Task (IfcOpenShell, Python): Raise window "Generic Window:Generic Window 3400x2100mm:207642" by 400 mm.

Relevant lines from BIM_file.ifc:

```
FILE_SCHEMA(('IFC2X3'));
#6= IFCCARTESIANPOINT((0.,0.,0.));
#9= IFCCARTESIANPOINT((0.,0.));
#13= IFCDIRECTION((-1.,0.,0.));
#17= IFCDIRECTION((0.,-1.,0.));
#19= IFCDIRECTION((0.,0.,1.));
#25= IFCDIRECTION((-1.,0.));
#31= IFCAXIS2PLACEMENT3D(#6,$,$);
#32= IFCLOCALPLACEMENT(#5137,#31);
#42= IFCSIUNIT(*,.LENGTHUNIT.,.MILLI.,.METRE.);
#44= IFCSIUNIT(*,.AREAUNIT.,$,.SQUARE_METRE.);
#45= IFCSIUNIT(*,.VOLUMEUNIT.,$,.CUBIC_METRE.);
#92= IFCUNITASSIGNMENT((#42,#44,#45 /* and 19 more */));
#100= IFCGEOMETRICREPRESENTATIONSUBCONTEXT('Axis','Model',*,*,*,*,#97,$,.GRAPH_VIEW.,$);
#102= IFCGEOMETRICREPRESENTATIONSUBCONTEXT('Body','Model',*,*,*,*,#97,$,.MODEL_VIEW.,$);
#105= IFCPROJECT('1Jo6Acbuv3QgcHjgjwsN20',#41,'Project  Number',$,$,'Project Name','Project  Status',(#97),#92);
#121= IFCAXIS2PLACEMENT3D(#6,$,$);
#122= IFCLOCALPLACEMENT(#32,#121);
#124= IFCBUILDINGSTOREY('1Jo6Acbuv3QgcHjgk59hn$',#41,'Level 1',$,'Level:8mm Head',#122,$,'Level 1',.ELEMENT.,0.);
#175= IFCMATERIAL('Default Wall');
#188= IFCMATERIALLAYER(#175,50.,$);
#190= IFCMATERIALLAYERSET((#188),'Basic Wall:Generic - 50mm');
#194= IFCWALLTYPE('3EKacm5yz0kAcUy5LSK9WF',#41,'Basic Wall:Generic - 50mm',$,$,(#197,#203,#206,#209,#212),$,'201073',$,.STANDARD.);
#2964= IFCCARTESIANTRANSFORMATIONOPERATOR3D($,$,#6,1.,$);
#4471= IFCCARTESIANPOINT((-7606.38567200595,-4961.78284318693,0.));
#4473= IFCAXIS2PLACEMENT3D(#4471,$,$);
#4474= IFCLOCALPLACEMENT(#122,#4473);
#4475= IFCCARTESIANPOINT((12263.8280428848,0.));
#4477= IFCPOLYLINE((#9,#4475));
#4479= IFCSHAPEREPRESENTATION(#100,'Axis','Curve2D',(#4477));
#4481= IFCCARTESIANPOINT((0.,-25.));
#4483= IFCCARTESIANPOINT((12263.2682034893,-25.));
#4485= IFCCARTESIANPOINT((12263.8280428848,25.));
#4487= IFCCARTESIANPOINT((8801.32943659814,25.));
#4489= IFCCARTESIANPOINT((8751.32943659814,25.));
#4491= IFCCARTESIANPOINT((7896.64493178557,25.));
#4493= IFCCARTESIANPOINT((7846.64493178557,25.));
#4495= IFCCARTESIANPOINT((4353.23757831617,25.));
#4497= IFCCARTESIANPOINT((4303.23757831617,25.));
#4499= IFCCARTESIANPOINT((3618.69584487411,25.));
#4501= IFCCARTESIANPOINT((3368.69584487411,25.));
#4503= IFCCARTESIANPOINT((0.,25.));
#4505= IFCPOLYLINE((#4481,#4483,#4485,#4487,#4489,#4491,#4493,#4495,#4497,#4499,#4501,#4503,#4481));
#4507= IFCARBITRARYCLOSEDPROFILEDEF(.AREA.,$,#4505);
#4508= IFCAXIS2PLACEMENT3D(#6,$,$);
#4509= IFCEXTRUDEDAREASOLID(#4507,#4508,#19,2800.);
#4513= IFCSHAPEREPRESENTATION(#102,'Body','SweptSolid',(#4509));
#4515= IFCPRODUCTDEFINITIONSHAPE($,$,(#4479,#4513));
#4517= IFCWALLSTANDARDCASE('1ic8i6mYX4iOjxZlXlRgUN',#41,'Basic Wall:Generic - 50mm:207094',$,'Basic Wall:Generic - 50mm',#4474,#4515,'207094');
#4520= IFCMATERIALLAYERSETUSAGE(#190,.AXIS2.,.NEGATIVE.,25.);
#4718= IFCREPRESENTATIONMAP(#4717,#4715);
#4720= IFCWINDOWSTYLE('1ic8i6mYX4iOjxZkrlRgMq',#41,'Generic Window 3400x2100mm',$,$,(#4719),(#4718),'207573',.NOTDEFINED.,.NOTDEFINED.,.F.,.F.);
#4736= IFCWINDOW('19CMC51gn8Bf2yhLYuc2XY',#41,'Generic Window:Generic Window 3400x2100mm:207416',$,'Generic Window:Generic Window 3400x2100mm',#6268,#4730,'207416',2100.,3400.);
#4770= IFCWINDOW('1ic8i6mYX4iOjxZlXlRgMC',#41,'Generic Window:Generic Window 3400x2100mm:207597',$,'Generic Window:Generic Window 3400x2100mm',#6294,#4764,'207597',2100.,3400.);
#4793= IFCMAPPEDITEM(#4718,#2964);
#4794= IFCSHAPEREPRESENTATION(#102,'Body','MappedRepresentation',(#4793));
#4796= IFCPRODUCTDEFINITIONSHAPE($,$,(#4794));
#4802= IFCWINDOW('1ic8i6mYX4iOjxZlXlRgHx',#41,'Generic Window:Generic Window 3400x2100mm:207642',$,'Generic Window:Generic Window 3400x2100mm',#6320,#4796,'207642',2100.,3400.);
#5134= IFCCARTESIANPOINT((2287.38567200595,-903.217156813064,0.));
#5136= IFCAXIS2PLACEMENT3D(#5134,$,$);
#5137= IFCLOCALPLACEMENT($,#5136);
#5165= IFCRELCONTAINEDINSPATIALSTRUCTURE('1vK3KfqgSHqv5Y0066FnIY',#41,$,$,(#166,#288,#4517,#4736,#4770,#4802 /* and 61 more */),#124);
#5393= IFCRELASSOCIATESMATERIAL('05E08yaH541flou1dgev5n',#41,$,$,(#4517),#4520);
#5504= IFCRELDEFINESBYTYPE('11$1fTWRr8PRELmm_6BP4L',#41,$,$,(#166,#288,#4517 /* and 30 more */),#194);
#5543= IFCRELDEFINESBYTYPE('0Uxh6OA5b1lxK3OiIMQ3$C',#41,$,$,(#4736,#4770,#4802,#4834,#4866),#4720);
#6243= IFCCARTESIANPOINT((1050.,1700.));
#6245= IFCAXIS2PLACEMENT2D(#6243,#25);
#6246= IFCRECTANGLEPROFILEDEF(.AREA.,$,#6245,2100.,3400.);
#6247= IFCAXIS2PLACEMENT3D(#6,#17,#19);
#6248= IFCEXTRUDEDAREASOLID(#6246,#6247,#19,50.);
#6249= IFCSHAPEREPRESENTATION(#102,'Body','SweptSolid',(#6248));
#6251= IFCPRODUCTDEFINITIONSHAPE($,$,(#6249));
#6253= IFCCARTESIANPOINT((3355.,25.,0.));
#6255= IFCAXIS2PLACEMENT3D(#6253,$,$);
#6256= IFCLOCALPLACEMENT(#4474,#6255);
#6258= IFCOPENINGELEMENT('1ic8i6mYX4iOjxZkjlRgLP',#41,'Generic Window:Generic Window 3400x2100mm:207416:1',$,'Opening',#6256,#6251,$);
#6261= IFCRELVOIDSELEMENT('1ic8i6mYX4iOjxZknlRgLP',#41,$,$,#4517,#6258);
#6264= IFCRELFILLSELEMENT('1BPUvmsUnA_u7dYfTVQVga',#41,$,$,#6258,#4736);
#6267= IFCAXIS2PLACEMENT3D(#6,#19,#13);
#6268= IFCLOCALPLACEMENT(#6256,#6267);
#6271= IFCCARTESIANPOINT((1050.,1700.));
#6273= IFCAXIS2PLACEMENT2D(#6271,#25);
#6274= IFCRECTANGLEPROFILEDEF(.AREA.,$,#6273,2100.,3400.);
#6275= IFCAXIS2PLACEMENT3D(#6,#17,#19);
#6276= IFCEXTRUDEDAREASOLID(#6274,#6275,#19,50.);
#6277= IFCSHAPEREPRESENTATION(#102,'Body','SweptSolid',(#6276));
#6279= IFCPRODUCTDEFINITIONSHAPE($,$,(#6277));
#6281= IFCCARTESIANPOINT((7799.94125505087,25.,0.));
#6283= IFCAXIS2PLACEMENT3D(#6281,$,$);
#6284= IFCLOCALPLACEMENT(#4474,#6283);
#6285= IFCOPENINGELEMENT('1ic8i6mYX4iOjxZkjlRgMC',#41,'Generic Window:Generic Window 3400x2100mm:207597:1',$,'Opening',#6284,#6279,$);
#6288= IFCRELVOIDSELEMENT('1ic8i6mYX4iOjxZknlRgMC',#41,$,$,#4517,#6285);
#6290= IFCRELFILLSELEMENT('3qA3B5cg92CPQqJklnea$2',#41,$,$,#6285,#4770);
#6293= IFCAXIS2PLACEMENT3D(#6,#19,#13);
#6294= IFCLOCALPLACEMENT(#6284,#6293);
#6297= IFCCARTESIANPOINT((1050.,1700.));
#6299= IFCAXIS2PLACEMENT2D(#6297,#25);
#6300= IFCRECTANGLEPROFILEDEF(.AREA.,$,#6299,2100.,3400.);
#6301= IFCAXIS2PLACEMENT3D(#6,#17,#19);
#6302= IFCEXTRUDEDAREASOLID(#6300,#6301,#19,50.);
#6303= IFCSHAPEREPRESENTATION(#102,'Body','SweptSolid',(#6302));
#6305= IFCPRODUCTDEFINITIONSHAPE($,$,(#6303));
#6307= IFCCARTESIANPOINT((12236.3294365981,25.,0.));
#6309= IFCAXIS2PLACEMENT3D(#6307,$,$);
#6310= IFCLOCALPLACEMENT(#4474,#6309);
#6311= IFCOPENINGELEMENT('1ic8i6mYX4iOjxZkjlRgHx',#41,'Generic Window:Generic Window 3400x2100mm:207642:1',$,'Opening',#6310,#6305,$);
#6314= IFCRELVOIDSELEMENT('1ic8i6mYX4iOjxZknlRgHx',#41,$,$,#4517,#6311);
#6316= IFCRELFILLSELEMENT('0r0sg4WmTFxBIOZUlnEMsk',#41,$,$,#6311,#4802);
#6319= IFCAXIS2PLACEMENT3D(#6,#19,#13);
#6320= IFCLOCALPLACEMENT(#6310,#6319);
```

```python
import numpy as np
import ifcopenshell
import ifcopenshell.api.geometry
import ifcopenshell.util.placement
import ifcopenshell.util.unit

model = ifcopenshell.open("BIM_file.ifc")
unit_scale = ifcopenshell.util.unit.calculate_unit_scale(model)

window = model.by_guid("1ic8i6mYX4iOjxZlXlRgHx")
opening = window.FillsVoids[0].RelatingOpeningElement
dz = 400.0

shift = np.array([0.0, 0.0, dz])
# The window is placed relative to its opening, so it follows when the opening moves.
matrix = ifcopenshell.util.placement.get_local_placement(opening.ObjectPlacement)
matrix[:3, 3] += shift
ifcopenshell.api.geometry.edit_object_placement(
    model, product=opening, matrix=matrix, is_si=False, should_transform_children=True
)

print(f"moved by {dz * unit_scale:+.3f} m")

model.write("BIM_file_edited.ifc")
```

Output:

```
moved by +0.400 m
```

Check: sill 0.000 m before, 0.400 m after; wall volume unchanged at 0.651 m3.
